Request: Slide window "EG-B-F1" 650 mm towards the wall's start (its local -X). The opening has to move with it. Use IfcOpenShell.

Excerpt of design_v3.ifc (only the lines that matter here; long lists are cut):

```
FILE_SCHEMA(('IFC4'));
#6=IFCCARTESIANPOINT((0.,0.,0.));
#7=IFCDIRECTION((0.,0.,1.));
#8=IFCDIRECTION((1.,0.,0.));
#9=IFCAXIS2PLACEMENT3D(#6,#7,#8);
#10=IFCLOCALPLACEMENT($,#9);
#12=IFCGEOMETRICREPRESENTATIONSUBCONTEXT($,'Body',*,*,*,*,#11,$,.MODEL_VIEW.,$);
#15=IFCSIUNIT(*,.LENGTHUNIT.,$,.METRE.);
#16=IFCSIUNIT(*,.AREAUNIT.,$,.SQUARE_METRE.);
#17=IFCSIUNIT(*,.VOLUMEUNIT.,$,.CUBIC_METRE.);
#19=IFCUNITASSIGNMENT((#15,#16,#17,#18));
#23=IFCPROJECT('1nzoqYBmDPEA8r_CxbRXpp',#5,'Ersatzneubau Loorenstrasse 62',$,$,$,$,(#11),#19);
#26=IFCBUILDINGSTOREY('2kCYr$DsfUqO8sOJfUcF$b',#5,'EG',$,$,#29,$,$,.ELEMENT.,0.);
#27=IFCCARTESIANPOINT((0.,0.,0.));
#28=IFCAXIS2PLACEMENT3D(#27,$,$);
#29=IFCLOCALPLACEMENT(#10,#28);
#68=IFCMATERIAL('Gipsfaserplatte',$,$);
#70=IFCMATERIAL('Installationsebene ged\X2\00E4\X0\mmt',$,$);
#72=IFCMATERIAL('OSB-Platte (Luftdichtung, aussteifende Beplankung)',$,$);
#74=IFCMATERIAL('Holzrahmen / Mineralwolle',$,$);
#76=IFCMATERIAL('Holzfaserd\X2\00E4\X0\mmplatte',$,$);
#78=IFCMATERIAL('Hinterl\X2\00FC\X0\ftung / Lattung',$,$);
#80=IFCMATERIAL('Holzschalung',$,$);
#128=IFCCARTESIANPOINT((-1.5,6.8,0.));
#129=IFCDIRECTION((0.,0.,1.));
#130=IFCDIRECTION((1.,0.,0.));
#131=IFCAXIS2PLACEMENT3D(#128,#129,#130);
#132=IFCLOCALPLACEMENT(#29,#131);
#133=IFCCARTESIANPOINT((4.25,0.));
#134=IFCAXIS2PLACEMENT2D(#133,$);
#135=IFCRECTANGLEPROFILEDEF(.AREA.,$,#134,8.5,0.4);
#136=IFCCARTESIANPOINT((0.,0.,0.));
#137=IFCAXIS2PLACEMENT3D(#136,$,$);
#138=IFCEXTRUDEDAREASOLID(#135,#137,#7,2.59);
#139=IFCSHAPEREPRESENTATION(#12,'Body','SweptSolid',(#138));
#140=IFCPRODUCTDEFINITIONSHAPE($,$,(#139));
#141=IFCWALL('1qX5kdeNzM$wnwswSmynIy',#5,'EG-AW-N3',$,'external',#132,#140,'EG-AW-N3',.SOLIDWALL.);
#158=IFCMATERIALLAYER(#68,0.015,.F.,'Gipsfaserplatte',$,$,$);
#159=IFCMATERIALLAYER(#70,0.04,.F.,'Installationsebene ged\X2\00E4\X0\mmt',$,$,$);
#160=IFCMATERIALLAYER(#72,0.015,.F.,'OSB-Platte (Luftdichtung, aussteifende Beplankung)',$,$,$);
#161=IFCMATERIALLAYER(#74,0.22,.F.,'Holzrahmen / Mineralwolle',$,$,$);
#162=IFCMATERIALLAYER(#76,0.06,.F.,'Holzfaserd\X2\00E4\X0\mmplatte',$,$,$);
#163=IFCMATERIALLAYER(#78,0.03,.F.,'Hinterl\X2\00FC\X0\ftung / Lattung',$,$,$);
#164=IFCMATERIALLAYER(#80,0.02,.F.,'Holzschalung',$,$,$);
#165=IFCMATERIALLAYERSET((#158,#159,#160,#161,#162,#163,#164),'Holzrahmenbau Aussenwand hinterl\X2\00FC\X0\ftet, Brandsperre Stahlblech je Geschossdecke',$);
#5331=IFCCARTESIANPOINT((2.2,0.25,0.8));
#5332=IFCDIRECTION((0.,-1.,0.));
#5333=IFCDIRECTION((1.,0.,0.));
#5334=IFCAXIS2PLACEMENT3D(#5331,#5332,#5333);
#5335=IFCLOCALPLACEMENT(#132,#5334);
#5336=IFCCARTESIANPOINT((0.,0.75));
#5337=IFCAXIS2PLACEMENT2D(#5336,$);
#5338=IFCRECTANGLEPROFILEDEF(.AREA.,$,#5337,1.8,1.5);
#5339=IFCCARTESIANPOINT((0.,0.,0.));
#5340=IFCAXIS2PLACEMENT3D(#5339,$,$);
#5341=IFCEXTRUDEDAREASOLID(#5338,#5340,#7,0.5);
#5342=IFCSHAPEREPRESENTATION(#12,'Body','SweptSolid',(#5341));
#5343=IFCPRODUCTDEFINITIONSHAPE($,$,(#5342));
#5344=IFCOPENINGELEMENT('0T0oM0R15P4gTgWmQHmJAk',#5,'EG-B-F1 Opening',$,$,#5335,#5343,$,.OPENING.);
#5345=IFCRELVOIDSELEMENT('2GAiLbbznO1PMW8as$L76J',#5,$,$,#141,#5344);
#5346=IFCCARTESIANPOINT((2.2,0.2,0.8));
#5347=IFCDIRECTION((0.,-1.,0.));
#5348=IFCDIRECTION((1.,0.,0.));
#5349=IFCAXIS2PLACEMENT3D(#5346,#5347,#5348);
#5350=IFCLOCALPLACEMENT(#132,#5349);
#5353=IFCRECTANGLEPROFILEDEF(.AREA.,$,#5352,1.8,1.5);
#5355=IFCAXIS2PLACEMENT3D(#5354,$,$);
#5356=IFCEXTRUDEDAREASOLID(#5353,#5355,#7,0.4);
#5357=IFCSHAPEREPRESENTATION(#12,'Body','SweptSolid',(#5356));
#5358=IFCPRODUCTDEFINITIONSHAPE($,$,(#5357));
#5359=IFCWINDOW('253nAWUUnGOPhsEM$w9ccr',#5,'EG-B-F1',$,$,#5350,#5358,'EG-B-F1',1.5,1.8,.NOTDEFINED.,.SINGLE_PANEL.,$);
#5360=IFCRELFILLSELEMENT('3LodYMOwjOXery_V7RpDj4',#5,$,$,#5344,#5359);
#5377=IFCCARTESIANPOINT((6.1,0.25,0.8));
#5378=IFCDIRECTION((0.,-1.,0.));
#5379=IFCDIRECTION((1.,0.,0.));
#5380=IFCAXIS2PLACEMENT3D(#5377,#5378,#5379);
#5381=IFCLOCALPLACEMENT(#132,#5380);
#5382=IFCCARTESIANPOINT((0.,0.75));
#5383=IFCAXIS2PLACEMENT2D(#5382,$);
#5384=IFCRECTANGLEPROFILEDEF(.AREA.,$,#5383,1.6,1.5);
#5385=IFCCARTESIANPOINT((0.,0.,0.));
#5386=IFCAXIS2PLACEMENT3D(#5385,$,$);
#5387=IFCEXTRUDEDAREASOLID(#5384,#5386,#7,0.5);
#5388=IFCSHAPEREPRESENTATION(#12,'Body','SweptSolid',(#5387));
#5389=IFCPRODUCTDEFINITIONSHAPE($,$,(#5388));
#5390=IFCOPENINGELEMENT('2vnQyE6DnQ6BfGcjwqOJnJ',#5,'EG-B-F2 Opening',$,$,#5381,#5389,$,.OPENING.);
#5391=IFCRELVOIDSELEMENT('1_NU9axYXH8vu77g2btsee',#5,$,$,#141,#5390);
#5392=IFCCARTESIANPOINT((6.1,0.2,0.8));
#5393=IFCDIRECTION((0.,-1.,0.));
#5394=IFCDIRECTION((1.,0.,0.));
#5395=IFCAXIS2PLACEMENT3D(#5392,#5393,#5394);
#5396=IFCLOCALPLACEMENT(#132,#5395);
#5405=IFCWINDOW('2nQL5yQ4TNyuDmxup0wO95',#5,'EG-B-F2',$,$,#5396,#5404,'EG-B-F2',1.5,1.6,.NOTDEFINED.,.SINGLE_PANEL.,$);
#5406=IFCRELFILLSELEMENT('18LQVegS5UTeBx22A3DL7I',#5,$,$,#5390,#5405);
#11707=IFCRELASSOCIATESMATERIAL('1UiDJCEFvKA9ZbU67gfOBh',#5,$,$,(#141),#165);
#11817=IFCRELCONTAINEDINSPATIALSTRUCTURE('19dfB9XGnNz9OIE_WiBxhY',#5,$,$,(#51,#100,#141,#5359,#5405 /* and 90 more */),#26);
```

```python
import ifcopenshell
import ifcopenshell.api.geometry
import ifcopenshell.util.placement
import ifcopenshell.util.unit

model = ifcopenshell.open("design_v3.ifc")
unit_scale = ifcopenshell.util.unit.calculate_unit_scale(model)

window = model.by_id(5359)
opening = window.FillsVoids[0].RelatingOpeningElement
wall = opening.VoidsElements[0].RelatingBuildingElement

wall_matrix = ifcopenshell.util.placement.get_local_placement(wall.ObjectPlacement)
shift = wall_matrix[:3, 0] * -0.65 / unit_scale
before = ifcopenshell.util.placement.get_local_placement(window.ObjectPlacement)[:3, 3].copy()

# The window is not placed relative to its opening, so move both.
for product in (opening, window):
    matrix = ifcopenshell.util.placement.get_local_placement(product.ObjectPlacement)
    matrix[:3, 3] += shift
    ifcopenshell.api.geometry.edit_object_placement(model, product=product, matrix=matrix, is_si=False)

after = ifcopenshell.util.placement.get_local_placement(window.ObjectPlacement)[:3, 3]
print("window moved by", (after - before).round(3) + 0.0)

model.write("design_v3_rev.ifc")
```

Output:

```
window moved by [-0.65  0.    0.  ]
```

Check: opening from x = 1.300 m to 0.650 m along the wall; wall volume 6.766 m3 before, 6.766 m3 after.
